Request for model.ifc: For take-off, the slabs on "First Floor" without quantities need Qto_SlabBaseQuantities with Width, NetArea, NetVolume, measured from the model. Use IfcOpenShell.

First a look at what the model holds.

```python
import ifcopenshell
import ifcopenshell.util.element
import ifcopenshell.util.unit

model = ifcopenshell.open("model.ifc")
print(model.schema)
for unit_type in ("LENGTHUNIT", "AREAUNIT", "VOLUMEUNIT"):
    print(unit_type, ifcopenshell.util.unit.calculate_unit_scale(model, unit_type))
storey = next(s for s in model.by_type("IfcBuildingStorey") if s.Name == "First Floor")
slabs = [e for e in ifcopenshell.util.element.get_decomposition(storey) if e.is_a("IfcSlab")]
for e in sorted(slabs, key=lambda e: e.id()):
    print(e.id(), e.is_a(), e.Name, list(ifcopenshell.util.element.get_psets(e, qtos_only=True)), sep=" | ")
```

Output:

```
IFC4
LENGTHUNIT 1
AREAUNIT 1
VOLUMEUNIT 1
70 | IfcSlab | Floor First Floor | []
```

```python
import ifcopenshell
import ifcopenshell.api.pset
import ifcopenshell.geom
import ifcopenshell.util.element
import ifcopenshell.util.shape
import ifcopenshell.util.unit

model = ifcopenshell.open("model.ifc")
unit_scale = ifcopenshell.util.unit.calculate_unit_scale(model)
area_scale = ifcopenshell.util.unit.calculate_unit_scale(model, "AREAUNIT")
volume_scale = ifcopenshell.util.unit.calculate_unit_scale(model, "VOLUMEUNIT")
settings = ifcopenshell.geom.settings()

storey = next(s for s in model.by_type("IfcBuildingStorey") if s.Name == "First Floor")
slabs = [e for e in ifcopenshell.util.element.get_decomposition(storey) if e.is_a("IfcSlab")]

for e in sorted(slabs, key=lambda e: e.id()):
    if ifcopenshell.util.element.get_psets(e, qtos_only=True, should_inherit=False):
        continue
    # Geometry comes back in metres, in the element's own axes.
    shape = ifcopenshell.geom.create_shape(settings, e)
    values = {
        "Width": ifcopenshell.util.shape.get_z(shape.geometry) / unit_scale,
        "NetArea": ifcopenshell.util.shape.get_footprint_area(shape.geometry) / area_scale,
        "NetVolume": ifcopenshell.util.shape.get_volume(shape.geometry) / volume_scale,
    }
    qto = ifcopenshell.api.pset.add_qto(model, product=e, name="Qto_SlabBaseQuantities")
    ifcopenshell.api.pset.edit_qto(model, qto=qto, properties=values)
    print(e.id(), {k: round(v, 3) for k, v in values.items()})

model.write("model-out.ifc")
```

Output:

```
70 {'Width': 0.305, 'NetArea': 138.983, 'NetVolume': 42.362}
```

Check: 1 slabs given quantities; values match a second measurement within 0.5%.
